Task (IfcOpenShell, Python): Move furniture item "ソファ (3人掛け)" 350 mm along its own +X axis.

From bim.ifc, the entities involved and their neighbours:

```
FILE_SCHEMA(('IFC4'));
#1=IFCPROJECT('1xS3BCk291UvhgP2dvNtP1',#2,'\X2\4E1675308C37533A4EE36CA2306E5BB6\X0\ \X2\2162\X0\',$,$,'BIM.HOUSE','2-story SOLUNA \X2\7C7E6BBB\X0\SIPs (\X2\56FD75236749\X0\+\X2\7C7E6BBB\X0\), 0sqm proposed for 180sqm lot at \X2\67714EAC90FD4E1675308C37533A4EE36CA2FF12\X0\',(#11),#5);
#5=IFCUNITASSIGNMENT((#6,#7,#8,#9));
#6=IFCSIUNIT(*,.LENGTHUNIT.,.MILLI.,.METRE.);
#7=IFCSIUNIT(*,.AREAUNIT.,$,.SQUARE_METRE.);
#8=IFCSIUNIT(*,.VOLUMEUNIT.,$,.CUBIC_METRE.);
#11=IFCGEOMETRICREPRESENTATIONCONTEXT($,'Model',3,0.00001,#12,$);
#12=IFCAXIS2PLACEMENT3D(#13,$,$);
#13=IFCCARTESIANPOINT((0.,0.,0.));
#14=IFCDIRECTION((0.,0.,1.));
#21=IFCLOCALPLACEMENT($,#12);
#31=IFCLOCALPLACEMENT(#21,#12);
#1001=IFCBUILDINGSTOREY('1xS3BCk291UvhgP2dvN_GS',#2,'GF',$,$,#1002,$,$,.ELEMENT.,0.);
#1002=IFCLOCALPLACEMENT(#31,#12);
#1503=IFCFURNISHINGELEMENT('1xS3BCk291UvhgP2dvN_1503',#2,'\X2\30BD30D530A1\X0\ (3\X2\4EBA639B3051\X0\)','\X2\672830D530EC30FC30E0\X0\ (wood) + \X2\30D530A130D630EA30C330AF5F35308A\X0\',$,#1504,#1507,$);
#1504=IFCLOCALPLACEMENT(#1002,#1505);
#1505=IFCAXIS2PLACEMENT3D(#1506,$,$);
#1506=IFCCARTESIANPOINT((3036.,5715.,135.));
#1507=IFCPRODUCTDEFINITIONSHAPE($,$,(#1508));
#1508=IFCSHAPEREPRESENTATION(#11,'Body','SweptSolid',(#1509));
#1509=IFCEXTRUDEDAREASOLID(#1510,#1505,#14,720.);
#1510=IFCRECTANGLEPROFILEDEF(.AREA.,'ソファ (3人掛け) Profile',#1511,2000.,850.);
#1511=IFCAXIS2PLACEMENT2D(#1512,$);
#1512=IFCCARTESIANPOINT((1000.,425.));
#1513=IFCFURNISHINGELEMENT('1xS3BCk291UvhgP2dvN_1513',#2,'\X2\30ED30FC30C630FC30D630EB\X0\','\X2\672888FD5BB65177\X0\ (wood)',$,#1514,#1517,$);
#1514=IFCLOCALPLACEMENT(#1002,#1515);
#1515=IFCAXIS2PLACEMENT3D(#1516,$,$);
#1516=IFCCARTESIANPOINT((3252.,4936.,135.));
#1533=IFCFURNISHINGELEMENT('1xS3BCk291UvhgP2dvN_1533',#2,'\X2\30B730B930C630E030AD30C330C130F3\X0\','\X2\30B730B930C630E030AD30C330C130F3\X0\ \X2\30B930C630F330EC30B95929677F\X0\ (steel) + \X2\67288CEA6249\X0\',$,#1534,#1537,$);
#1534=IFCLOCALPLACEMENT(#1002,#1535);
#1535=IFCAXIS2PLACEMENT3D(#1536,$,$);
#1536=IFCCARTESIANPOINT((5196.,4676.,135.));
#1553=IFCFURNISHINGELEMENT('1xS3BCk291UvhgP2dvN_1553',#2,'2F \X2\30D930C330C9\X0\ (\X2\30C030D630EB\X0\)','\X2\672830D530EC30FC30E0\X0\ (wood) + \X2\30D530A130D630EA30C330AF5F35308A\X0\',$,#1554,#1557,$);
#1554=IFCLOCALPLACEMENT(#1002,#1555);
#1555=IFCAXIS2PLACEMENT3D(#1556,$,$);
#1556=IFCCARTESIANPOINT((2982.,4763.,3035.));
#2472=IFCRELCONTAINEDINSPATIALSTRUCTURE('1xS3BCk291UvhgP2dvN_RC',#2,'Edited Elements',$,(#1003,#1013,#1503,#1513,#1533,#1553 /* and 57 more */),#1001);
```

```python
import ifcopenshell
import ifcopenshell.api.geometry
import ifcopenshell.util.placement
import ifcopenshell.util.unit

model = ifcopenshell.open("bim.ifc")
unit_scale = ifcopenshell.util.unit.calculate_unit_scale(model)

item = model.by_guid("1xS3BCk291UvhgP2dvN_1503")
matrix = ifcopenshell.util.placement.get_local_placement(item.ObjectPlacement)
matrix[:3, 3] += matrix[:3, 0] * 0.35 / unit_scale
ifcopenshell.api.geometry.edit_object_placement(model, product=item, matrix=matrix, is_si=False)

print(ifcopenshell.util.placement.get_local_placement(item.ObjectPlacement).round(3) + 0.0)

model.write("bim_updated.ifc")
```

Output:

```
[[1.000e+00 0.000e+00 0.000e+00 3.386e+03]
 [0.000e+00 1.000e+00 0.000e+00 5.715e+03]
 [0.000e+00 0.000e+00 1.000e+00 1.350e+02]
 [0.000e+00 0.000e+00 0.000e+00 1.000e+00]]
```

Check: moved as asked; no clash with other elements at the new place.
